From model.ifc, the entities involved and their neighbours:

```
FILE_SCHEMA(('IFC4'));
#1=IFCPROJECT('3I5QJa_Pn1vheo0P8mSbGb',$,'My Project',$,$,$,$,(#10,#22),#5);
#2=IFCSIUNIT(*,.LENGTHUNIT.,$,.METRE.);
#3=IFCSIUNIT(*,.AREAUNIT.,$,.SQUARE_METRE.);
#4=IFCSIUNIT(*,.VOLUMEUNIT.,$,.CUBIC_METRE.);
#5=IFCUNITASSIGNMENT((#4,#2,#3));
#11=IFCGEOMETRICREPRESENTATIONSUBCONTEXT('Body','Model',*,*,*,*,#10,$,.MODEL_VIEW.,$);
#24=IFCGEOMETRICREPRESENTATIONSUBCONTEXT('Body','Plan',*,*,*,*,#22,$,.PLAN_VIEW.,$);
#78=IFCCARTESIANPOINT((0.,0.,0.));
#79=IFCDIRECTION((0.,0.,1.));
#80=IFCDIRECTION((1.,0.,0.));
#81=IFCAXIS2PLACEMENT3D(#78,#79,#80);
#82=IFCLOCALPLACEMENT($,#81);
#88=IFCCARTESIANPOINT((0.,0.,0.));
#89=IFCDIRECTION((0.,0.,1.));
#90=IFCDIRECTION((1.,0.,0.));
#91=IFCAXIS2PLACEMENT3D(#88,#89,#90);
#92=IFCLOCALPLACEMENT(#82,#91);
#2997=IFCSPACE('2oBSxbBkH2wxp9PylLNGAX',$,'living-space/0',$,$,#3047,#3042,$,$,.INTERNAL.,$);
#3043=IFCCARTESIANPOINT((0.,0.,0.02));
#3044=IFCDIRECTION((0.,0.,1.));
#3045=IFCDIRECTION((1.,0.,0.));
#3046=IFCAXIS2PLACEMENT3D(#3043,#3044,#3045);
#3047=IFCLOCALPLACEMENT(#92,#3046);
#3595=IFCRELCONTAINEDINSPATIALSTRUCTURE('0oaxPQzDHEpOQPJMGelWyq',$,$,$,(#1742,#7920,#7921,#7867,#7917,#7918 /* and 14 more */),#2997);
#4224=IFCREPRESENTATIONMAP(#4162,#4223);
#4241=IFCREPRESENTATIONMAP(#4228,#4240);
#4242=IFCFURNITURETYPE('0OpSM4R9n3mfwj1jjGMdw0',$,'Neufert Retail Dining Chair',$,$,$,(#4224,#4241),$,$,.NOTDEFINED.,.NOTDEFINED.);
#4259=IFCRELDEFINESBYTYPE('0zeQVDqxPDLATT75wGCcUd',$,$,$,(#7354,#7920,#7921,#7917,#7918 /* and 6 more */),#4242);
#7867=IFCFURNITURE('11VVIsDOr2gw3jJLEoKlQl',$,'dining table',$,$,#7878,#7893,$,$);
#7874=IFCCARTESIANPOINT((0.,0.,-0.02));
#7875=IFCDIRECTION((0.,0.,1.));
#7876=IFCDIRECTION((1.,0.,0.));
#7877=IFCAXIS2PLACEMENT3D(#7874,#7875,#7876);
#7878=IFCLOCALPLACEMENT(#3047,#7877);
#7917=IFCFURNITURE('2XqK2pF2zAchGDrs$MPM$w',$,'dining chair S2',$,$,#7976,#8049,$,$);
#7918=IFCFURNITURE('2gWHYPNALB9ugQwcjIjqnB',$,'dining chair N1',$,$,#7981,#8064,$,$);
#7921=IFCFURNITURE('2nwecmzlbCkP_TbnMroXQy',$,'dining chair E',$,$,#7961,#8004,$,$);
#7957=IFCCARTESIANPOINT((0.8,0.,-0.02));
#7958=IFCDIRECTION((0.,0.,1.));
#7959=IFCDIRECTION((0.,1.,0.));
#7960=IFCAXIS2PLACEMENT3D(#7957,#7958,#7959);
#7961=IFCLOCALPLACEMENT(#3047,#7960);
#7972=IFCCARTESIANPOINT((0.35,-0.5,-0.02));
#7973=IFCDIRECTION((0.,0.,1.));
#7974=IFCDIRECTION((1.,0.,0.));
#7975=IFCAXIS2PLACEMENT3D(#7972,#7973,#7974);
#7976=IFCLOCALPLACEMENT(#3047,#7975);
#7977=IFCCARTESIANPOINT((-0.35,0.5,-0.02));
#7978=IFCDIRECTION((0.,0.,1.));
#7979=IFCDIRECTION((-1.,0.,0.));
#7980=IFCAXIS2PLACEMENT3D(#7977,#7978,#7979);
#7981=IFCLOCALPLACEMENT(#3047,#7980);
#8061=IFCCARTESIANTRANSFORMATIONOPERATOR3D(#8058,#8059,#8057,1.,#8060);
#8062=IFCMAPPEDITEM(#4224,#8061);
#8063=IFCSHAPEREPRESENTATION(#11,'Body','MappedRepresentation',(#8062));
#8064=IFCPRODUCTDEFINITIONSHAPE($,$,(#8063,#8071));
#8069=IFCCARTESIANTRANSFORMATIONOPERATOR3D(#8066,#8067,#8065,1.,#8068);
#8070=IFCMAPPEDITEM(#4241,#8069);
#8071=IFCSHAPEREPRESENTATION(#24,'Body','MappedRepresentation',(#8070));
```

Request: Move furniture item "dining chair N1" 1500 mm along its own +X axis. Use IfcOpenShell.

```python
import ifcopenshell
import ifcopenshell.api.geometry
import ifcopenshell.util.placement

model = ifcopenshell.open("model.ifc")

item = model.by_guid("2gWHYPNALB9ugQwcjIjqnB")
matrix = ifcopenshell.util.placement.get_local_placement(item.ObjectPlacement)
matrix[:3, 3] += matrix[:3, 0] * 1.5
ifcopenshell.api.geometry.edit_object_placement(model, product=item, matrix=matrix, is_si=False)

print(ifcopenshell.util.placement.get_local_placement(item.ObjectPlacement).round(3) + 0.0)

model.write("model_v2.ifc")
```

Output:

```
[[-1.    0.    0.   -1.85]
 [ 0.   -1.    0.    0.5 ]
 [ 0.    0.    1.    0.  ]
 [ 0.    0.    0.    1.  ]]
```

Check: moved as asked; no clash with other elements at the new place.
